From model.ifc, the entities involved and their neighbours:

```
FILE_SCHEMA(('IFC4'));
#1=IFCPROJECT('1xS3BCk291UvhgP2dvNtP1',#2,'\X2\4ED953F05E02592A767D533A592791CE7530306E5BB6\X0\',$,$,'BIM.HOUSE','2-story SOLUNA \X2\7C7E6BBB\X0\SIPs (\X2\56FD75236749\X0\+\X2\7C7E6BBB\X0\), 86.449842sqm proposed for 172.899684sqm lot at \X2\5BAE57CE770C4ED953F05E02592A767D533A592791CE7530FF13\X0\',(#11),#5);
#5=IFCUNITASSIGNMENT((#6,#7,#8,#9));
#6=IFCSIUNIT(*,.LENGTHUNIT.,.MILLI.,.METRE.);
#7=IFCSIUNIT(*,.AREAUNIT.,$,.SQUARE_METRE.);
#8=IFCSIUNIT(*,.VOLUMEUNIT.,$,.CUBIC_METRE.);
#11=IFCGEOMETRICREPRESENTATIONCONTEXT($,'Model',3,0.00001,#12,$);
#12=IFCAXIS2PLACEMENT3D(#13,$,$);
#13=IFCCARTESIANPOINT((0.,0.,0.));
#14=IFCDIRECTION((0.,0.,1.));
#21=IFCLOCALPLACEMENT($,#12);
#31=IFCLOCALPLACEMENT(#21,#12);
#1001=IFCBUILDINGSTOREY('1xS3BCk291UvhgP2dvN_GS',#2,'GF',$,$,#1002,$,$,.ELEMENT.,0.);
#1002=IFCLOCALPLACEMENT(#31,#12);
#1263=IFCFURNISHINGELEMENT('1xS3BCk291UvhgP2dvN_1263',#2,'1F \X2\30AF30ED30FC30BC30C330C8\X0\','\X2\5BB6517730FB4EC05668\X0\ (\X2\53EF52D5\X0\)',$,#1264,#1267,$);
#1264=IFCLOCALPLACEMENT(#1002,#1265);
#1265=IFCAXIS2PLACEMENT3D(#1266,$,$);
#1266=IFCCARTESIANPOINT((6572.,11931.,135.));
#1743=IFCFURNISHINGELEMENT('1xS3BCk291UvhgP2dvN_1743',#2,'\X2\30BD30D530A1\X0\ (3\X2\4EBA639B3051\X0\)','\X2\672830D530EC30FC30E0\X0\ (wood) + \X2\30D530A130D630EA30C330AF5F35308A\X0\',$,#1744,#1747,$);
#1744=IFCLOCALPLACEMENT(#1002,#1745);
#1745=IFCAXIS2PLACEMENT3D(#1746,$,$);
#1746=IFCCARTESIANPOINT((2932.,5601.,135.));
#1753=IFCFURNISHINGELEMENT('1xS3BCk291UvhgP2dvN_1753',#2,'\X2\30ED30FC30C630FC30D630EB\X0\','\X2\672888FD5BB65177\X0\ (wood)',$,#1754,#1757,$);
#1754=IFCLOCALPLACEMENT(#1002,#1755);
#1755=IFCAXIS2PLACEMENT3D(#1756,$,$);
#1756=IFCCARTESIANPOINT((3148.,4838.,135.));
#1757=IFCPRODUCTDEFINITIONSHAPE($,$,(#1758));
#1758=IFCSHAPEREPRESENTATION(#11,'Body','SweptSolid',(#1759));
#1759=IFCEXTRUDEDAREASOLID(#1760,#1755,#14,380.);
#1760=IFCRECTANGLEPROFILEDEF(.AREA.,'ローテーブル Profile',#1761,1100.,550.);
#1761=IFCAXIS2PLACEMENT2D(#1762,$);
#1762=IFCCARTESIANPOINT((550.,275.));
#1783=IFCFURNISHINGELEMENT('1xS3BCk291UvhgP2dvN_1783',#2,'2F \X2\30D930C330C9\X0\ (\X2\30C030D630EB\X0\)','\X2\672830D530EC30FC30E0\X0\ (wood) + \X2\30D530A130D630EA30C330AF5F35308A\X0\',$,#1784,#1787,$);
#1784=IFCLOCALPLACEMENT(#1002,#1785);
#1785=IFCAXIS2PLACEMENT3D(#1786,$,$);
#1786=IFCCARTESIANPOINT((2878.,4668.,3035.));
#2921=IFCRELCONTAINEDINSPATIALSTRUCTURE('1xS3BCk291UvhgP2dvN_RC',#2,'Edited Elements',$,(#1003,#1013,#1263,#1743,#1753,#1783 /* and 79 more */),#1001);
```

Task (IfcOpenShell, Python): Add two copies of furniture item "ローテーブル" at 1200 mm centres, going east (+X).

```python
import numpy as np
import ifcopenshell
import ifcopenshell.api.geometry
import ifcopenshell.api.root
import ifcopenshell.util.element
import ifcopenshell.util.placement
import ifcopenshell.util.unit

model = ifcopenshell.open("model.ifc")
unit_scale = ifcopenshell.util.unit.calculate_unit_scale(model)


def reuse_history(source, copy):
    """copy_class also copies each property set's owner history, people and application; keep the originals."""
    for rel in copy.IsDefinedBy:
        if rel.is_a("IfcRelDefinesByProperties") and (history := rel.RelatingPropertyDefinition.OwnerHistory):
            rel.RelatingPropertyDefinition.OwnerHistory = source.OwnerHistory
            ifcopenshell.util.element.remove_deep2(model, history)


source = model.by_guid("1xS3BCk291UvhgP2dvN_1753")
base = ifcopenshell.util.placement.get_local_placement(source.ObjectPlacement)
step = np.array([1.0, 0.0, 0.0]) * 1.2 / unit_scale

for i in range(1, 3):
    copy = ifcopenshell.api.root.copy_class(model, product=source)
    copy.Representation = ifcopenshell.util.element.copy_deep(
        model, source.Representation, exclude=["IfcGeometricRepresentationContext", "IfcRepresentationMap"]
    )
    reuse_history(source, copy)
    matrix = base.copy()
    matrix[:3, 3] += i * step
    print("added at", matrix[:3, 3].round(3) + 0.0)
    ifcopenshell.api.geometry.edit_object_placement(model, product=copy, matrix=matrix, is_si=False)

model.write("model_updated.ifc")
```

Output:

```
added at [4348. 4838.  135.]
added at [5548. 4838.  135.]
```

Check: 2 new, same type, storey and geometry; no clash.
